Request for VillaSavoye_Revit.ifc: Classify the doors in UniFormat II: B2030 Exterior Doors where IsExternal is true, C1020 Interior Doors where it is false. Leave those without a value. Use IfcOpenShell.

First a look at what the model holds.

```python
import ifcopenshell
import ifcopenshell.util.element

model = ifcopenshell.open("VillaSavoye_Revit.ifc")
print(model.schema)
print("classifications:", [c.Name for c in model.by_type("IfcClassification")])
values = [ifcopenshell.util.element.get_pset(e, "Pset_DoorCommon", "IsExternal") for e in model.by_type("IfcDoor")]
for value in (True, False, None):
    print("IsExternal", value, values.count(value))
```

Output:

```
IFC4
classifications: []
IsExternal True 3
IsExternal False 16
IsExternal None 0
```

```python
import ifcopenshell
import ifcopenshell.api.classification
import ifcopenshell.util.element

model = ifcopenshell.open("VillaSavoye_Revit.ifc")

system = ifcopenshell.api.classification.add_classification(model, classification="UniFormat II")

doors = model.by_type("IfcDoor")
external = {e: ifcopenshell.util.element.get_pset(e, "Pset_DoorCommon", "IsExternal") for e in doors}
for flag, code, name in ((True, "B2030", "Exterior Doors"), (False, "C1020", "Interior Doors")):
    products = [e for e in doors if external[e] is flag]
    ifcopenshell.api.classification.add_reference(
        model, products=products, classification=system, identification=code, name=name
    )
    print(code, len(products))

model.write("VillaSavoye_Revit_updated.ifc")
```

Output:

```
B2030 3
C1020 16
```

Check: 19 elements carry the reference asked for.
